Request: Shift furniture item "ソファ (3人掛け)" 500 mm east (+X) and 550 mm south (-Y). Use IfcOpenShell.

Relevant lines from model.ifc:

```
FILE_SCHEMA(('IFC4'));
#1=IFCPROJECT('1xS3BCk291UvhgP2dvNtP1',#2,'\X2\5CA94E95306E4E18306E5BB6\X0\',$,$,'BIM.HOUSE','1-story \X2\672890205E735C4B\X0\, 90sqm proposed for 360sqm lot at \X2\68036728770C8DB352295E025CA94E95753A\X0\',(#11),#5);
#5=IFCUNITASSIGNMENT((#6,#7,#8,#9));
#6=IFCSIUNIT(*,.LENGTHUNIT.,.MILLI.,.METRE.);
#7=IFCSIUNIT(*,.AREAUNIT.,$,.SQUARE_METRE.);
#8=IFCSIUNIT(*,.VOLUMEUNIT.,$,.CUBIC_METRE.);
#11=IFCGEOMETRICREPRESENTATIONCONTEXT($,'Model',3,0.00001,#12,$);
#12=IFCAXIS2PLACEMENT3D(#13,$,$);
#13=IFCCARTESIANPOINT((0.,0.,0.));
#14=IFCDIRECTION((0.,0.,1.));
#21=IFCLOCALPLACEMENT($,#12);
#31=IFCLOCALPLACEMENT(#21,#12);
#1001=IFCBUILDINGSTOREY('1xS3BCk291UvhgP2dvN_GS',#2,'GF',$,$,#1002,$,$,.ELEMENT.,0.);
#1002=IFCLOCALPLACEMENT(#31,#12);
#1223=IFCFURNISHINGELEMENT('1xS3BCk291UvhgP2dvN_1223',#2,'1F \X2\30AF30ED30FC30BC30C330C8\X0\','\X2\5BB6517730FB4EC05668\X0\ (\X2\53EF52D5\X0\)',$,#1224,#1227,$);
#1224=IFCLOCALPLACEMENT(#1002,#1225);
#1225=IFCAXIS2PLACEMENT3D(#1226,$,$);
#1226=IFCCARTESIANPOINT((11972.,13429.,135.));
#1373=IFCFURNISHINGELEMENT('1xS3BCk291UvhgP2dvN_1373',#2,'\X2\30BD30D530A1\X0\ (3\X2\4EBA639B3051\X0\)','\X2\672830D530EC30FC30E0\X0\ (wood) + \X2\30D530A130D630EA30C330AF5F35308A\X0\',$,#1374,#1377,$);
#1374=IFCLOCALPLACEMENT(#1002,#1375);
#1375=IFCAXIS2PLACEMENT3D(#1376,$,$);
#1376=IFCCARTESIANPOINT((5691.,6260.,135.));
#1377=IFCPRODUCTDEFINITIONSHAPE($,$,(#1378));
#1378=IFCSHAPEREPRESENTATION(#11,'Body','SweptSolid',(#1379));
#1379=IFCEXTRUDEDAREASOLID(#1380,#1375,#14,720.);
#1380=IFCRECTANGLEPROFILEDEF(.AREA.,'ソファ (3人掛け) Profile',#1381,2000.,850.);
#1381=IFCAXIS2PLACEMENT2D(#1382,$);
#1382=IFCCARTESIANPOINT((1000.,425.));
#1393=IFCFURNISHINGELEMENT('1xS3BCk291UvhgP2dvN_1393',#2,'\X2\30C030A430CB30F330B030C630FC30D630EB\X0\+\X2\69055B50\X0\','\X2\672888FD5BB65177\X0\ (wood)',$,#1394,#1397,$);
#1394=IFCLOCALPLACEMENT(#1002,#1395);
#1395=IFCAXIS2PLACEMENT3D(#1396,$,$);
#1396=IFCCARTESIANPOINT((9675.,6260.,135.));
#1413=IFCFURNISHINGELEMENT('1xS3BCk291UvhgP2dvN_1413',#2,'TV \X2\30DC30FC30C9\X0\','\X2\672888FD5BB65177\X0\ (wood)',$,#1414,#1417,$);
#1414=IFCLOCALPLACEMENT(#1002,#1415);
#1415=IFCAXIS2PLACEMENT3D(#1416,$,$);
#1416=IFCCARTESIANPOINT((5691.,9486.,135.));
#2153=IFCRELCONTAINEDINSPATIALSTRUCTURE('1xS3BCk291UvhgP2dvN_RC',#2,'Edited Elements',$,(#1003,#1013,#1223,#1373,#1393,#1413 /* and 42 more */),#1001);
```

```python
import ifcopenshell
import ifcopenshell.api.geometry
import ifcopenshell.util.placement
import ifcopenshell.util.unit

model = ifcopenshell.open("model.ifc")
unit_scale = ifcopenshell.util.unit.calculate_unit_scale(model)

item = model.by_guid("1xS3BCk291UvhgP2dvN_1373")
matrix = ifcopenshell.util.placement.get_local_placement(item.ObjectPlacement)
matrix[0, 3] += 0.5 / unit_scale
matrix[1, 3] -= 0.55 / unit_scale
ifcopenshell.api.geometry.edit_object_placement(model, product=item, matrix=matrix, is_si=False)

print(ifcopenshell.util.placement.get_local_placement(item.ObjectPlacement).round(3) + 0.0)

model.write("model-out.ifc")
```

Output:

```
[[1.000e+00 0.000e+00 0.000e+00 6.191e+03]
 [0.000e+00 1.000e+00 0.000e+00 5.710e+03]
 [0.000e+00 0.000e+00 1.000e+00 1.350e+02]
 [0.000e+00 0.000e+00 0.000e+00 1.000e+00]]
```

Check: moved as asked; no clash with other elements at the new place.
